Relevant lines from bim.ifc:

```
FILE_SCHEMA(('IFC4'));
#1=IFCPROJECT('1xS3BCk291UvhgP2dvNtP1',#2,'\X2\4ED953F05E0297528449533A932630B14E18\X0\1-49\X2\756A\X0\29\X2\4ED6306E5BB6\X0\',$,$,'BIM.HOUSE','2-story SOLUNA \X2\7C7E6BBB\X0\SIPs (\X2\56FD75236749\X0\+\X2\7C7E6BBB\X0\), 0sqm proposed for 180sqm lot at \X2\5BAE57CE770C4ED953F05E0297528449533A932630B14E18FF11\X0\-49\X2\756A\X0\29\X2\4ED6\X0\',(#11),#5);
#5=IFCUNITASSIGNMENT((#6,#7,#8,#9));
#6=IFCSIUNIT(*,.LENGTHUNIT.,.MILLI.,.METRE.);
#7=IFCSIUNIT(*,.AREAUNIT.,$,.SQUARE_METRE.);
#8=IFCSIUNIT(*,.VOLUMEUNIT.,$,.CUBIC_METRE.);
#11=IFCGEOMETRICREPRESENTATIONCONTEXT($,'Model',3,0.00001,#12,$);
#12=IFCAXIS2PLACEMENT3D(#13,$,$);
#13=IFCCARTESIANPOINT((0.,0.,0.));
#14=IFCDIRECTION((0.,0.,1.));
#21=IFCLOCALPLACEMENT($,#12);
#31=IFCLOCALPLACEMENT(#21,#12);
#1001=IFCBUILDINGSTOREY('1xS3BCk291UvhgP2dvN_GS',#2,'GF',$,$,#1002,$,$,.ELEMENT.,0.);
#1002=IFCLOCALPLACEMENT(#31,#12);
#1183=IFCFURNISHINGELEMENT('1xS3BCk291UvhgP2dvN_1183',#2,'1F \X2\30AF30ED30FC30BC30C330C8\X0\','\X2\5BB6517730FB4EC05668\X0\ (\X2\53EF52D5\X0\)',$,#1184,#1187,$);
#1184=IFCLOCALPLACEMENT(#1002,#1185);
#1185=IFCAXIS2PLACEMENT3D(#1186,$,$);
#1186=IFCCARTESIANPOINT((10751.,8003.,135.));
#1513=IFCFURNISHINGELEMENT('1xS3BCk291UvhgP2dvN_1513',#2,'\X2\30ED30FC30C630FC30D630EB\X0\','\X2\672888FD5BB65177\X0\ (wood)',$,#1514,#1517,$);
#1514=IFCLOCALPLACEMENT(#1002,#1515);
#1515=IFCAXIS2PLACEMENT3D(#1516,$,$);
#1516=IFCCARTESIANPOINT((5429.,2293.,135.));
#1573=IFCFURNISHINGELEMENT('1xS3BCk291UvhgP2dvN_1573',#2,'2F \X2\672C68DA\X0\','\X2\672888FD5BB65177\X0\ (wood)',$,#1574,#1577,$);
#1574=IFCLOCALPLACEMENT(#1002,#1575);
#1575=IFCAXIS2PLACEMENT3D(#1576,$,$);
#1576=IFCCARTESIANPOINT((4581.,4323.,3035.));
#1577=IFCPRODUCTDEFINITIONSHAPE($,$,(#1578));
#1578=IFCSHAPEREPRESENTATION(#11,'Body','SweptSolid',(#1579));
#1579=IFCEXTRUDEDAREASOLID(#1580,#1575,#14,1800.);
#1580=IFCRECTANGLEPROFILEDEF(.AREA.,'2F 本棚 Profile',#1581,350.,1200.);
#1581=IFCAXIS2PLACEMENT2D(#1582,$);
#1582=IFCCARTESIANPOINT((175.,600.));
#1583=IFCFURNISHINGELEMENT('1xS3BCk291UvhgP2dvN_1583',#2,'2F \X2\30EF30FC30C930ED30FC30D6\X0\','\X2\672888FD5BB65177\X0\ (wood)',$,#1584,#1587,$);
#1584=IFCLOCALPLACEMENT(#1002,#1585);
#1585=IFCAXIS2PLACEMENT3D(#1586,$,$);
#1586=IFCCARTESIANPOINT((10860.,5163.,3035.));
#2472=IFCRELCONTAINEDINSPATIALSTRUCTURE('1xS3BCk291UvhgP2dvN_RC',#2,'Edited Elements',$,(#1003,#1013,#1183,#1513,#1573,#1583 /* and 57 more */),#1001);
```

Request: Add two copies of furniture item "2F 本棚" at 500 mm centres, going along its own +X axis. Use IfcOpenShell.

```python
import ifcopenshell
import ifcopenshell.api.geometry
import ifcopenshell.api.root
import ifcopenshell.util.element
import ifcopenshell.util.placement

model = ifcopenshell.open("bim.ifc")


def reuse_history(source, copy):
    """copy_class also copies each property set's owner history, people and application; keep the originals."""
    for rel in copy.IsDefinedBy:
        if rel.is_a("IfcRelDefinesByProperties") and (history := rel.RelatingPropertyDefinition.OwnerHistory):
            rel.RelatingPropertyDefinition.OwnerHistory = source.OwnerHistory
            ifcopenshell.util.element.remove_deep2(model, history)


source = model.by_guid("1xS3BCk291UvhgP2dvN_1573")
base = ifcopenshell.util.placement.get_local_placement(source.ObjectPlacement)
step = base[:3, 0] * 500.0

for i in range(1, 3):
    copy = ifcopenshell.api.root.copy_class(model, product=source)
    copy.Representation = ifcopenshell.util.element.copy_deep(
        model, source.Representation, exclude=["IfcGeometricRepresentationContext", "IfcRepresentationMap"]
    )
    reuse_history(source, copy)
    matrix = base.copy()
    matrix[:3, 3] += i * step
    print("added at", matrix[:3, 3].round(3) + 0.0)
    ifcopenshell.api.geometry.edit_object_placement(model, product=copy, matrix=matrix, is_si=False)

model.write("bim_updated.ifc")
```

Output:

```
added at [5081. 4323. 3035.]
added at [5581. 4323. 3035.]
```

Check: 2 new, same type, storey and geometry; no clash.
